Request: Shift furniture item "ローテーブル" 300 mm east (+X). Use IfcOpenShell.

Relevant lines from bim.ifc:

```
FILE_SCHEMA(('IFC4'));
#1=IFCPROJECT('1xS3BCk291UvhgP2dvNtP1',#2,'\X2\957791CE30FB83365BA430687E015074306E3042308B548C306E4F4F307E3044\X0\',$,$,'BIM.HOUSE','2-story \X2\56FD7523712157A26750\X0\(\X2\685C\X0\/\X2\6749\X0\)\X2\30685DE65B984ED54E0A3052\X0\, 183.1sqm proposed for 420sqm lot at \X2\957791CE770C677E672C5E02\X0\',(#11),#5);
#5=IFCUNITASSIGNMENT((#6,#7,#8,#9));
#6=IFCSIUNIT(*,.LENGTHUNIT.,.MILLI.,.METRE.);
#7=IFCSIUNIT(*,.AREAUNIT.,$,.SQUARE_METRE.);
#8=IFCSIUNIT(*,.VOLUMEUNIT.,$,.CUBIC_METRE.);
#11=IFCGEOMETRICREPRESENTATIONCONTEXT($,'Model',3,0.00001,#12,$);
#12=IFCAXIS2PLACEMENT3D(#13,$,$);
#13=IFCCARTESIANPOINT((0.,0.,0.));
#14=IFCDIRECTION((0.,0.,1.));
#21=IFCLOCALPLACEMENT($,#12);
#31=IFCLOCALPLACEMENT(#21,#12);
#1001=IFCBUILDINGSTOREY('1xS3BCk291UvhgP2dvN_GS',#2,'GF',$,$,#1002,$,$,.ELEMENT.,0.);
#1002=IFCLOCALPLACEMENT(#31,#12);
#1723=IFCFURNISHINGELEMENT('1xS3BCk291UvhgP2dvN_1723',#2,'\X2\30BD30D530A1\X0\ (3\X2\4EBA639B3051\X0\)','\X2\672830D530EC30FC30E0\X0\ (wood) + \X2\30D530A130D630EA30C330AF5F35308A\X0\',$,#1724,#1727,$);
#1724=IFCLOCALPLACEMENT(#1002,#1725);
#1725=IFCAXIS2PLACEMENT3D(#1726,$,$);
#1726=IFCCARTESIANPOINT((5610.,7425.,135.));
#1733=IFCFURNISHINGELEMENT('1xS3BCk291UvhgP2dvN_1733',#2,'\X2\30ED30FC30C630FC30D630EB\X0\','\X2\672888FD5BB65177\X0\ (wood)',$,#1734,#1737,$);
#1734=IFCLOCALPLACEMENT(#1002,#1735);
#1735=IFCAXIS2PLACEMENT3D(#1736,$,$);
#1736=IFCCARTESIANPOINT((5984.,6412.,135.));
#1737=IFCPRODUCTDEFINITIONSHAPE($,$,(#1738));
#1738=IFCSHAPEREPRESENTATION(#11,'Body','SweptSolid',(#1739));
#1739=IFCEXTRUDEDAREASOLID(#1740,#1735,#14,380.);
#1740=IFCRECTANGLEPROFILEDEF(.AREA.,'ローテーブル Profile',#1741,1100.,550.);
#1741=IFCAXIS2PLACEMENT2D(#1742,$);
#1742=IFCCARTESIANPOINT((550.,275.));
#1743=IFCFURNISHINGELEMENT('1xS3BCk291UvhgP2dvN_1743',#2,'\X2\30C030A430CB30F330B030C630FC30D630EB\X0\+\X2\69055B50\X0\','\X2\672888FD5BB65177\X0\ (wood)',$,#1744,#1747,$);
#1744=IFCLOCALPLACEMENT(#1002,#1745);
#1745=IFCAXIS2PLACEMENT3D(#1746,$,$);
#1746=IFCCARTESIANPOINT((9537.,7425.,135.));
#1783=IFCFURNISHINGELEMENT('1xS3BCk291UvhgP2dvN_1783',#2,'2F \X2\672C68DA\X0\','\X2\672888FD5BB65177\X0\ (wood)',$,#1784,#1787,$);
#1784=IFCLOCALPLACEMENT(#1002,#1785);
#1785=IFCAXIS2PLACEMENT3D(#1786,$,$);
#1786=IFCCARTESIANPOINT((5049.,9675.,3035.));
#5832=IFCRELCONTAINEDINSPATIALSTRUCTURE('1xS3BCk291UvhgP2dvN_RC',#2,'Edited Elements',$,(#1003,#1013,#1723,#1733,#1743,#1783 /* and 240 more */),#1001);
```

```python
import ifcopenshell
import ifcopenshell.api.geometry
import ifcopenshell.util.placement

model = ifcopenshell.open("bim.ifc")

item = model.by_guid("1xS3BCk291UvhgP2dvN_1733")
matrix = ifcopenshell.util.placement.get_local_placement(item.ObjectPlacement)
matrix[0, 3] += 300.0
ifcopenshell.api.geometry.edit_object_placement(model, product=item, matrix=matrix, is_si=False)

print(ifcopenshell.util.placement.get_local_placement(item.ObjectPlacement).round(3) + 0.0)

model.write("bim_edited.ifc")
```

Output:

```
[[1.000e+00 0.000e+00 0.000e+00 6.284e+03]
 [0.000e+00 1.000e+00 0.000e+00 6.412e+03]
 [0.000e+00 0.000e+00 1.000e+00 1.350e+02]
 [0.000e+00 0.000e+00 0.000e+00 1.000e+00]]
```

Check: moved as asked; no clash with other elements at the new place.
